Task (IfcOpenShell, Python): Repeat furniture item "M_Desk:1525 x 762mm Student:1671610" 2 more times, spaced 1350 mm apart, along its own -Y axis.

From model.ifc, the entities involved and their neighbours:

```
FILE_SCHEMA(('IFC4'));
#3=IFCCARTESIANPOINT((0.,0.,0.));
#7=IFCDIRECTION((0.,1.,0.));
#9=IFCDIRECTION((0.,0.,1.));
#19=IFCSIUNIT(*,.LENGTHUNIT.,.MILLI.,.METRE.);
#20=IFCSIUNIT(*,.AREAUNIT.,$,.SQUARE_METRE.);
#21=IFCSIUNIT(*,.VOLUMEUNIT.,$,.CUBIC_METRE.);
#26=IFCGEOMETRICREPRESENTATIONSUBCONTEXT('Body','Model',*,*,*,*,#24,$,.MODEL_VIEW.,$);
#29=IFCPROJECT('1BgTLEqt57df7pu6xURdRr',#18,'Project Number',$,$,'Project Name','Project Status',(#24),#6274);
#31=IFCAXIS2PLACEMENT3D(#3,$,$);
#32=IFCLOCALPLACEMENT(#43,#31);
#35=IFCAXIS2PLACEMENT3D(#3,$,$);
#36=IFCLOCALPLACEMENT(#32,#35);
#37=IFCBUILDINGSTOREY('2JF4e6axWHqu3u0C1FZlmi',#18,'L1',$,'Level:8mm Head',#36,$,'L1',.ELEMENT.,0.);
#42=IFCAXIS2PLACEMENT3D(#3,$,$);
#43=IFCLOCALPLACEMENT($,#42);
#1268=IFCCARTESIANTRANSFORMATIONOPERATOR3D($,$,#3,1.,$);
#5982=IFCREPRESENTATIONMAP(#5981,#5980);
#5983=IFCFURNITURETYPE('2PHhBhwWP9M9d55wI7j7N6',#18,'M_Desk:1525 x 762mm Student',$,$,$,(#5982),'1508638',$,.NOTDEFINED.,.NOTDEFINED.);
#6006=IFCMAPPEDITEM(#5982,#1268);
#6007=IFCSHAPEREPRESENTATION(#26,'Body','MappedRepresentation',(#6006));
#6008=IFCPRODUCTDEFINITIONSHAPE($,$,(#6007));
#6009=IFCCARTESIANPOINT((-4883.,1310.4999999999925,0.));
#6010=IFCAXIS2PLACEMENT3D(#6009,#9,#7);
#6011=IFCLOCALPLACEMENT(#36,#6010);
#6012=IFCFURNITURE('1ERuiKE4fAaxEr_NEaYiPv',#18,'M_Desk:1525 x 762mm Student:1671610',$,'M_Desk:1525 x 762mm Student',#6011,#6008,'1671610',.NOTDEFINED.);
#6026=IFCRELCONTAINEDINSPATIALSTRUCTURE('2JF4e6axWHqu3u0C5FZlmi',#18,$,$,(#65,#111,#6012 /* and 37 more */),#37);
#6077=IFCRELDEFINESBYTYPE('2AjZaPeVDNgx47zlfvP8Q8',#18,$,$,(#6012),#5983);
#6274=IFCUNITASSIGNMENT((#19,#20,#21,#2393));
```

```python
import ifcopenshell
import ifcopenshell.api.geometry
import ifcopenshell.api.root
import ifcopenshell.util.element
import ifcopenshell.util.placement
import ifcopenshell.util.unit

model = ifcopenshell.open("model.ifc")
unit_scale = ifcopenshell.util.unit.calculate_unit_scale(model)


def reuse_history(source, copy):
    """copy_class also copies each property set's owner history, people and application; keep the originals."""
    for rel in copy.IsDefinedBy:
        if rel.is_a("IfcRelDefinesByProperties") and (history := rel.RelatingPropertyDefinition.OwnerHistory):
            rel.RelatingPropertyDefinition.OwnerHistory = source.OwnerHistory
            ifcopenshell.util.element.remove_deep2(model, history)


source = model.by_guid("1ERuiKE4fAaxEr_NEaYiPv")
base = ifcopenshell.util.placement.get_local_placement(source.ObjectPlacement)
step = -base[:3, 1] * 1.35 / unit_scale

for i in range(1, 3):
    copy = ifcopenshell.api.root.copy_class(model, product=source)
    copy.Representation = ifcopenshell.util.element.copy_deep(
        model, source.Representation, exclude=["IfcGeometricRepresentationContext", "IfcRepresentationMap"]
    )
    copy.Name = "M_Desk:1525 x 762mm Student"
    copy.Tag = None
    reuse_history(source, copy)
    matrix = base.copy()
    matrix[:3, 3] += i * step
    print("added at", matrix[:3, 3].round(3) + 0.0)
    ifcopenshell.api.geometry.edit_object_placement(model, product=copy, matrix=matrix, is_si=False)

model.write("model_updated.ifc")
```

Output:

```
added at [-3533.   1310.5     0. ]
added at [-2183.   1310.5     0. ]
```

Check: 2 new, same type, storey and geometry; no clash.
